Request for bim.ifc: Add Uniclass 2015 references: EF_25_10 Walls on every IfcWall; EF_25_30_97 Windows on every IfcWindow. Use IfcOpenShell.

First a look at what the model holds.

```python
import ifcopenshell

model = ifcopenshell.open("bim.ifc")
print(model.schema)
print("classifications:", [c.Name for c in model.by_type("IfcClassification")])
for ifc_class in ("IfcDoor", "IfcRoof", "IfcStair", "IfcWall", "IfcWindow"):
    print(ifc_class, len(model.by_type(ifc_class)))
```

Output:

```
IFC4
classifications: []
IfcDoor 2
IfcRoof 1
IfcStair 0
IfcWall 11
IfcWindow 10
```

```python
import ifcopenshell
import ifcopenshell.api.classification

model = ifcopenshell.open("bim.ifc")

system = ifcopenshell.api.classification.add_classification(model, classification="Uniclass 2015")

codes = {
    "IfcWall": ("EF_25_10", "Walls"),
    "IfcWindow": ("EF_25_30_97", "Windows"),
}
for ifc_class, (code, name) in codes.items():
    products = model.by_type(ifc_class)
    ifcopenshell.api.classification.add_reference(
        model, products=products, classification=system, identification=code, name=name
    )
    print(code, len(products))

model.write("bim_updated.ifc")
```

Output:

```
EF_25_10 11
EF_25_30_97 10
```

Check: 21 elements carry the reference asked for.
